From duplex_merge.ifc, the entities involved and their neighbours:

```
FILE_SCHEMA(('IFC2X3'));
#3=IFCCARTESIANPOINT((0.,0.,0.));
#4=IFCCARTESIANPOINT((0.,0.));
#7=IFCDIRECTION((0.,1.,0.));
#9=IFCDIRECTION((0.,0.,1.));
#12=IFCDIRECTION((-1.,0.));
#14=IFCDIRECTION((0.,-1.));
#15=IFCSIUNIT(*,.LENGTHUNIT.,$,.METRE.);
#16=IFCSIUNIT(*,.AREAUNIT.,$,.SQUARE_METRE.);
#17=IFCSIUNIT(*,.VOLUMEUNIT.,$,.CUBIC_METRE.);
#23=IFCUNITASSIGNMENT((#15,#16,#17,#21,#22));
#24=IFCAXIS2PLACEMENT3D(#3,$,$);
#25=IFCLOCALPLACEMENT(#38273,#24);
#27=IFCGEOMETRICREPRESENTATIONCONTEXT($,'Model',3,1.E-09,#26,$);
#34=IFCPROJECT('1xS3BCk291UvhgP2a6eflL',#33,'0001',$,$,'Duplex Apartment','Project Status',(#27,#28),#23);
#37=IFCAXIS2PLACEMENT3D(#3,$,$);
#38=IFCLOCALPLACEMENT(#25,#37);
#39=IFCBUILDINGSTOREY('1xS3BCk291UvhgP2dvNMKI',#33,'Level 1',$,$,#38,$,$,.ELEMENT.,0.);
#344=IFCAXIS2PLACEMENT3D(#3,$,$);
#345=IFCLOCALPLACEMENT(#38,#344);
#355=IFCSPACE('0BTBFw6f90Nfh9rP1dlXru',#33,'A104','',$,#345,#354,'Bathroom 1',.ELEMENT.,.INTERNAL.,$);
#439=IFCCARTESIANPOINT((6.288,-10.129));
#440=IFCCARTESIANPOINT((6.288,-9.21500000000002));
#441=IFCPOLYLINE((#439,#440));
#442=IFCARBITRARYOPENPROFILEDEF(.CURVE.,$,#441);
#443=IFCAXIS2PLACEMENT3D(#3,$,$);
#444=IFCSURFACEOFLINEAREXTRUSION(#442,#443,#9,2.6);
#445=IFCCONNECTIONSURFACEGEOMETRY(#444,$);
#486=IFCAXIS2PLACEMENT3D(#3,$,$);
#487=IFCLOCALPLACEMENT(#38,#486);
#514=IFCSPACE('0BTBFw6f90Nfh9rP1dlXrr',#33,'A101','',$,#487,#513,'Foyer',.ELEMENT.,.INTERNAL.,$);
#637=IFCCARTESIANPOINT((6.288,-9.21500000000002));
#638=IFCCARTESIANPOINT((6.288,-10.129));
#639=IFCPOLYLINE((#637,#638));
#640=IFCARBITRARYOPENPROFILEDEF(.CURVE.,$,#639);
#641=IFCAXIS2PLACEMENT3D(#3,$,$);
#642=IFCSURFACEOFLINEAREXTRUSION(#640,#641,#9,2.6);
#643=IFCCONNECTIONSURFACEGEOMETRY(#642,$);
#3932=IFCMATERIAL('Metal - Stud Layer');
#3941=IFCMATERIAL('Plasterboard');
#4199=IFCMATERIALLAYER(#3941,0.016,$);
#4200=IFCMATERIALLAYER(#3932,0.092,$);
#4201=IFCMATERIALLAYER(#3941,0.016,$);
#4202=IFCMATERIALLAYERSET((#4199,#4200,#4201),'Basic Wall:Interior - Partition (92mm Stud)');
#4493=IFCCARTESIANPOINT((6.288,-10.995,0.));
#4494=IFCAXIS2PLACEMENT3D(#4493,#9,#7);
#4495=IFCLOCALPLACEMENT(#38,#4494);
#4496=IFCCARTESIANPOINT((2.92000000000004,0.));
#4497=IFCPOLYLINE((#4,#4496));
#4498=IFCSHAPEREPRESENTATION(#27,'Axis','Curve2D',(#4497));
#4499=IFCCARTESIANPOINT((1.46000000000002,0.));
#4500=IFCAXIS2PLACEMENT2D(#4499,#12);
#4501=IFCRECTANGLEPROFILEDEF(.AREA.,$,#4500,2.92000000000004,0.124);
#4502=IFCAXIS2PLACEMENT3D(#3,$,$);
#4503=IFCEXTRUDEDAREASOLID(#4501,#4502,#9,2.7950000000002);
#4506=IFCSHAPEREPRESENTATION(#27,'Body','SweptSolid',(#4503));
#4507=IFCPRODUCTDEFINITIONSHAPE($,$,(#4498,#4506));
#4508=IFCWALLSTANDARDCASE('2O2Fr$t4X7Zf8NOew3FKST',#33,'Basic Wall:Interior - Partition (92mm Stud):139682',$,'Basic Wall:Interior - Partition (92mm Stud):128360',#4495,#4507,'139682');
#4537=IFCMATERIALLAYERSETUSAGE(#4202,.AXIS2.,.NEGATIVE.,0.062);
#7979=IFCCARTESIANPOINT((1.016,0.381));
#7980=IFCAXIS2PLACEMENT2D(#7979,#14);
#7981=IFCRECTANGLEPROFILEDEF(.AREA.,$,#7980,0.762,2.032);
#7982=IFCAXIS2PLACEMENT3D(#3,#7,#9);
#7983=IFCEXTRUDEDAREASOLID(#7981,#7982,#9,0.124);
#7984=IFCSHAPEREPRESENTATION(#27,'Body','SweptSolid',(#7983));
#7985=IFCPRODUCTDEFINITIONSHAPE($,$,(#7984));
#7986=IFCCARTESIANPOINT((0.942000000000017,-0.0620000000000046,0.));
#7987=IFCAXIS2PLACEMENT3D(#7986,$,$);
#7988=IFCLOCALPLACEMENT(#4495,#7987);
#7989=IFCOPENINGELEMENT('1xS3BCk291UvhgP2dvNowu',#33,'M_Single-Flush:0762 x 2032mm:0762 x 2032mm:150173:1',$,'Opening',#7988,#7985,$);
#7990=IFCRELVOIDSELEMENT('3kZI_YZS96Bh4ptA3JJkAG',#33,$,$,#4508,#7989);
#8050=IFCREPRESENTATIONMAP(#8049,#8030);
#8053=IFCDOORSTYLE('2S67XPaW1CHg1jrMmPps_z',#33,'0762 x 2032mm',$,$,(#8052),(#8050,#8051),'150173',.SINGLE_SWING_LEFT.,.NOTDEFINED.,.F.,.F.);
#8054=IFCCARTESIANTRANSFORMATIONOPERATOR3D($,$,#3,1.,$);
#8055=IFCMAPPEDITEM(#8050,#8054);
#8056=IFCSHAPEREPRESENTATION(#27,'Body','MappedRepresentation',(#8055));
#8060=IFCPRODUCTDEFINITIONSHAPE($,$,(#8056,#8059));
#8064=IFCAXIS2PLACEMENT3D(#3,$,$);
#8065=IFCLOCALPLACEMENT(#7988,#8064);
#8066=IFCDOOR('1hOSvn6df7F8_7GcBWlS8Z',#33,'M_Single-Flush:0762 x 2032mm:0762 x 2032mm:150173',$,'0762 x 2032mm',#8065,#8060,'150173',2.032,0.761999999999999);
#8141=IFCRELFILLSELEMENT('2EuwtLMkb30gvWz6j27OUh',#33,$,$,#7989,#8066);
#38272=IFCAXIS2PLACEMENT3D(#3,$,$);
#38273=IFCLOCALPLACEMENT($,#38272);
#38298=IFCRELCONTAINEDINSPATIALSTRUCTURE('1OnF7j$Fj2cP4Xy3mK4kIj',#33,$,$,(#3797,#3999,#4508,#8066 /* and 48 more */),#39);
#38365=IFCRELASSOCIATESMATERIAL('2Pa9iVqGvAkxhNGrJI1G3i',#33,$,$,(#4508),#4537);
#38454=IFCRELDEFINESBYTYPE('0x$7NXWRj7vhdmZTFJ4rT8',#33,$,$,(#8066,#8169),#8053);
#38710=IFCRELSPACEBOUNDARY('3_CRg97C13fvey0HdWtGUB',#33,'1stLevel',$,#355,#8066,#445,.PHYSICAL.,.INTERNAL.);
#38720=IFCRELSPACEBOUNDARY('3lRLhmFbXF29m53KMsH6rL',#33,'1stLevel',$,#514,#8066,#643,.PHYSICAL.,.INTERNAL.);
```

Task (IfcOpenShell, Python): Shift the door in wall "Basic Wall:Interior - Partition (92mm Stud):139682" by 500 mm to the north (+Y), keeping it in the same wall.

```python
import numpy as np
import ifcopenshell
import ifcopenshell.api.geometry
import ifcopenshell.util.placement

model = ifcopenshell.open("duplex_merge.ifc")

door = model.by_guid("1hOSvn6df7F8_7GcBWlS8Z")
opening = door.FillsVoids[0].RelatingOpeningElement
wall = opening.VoidsElements[0].RelatingBuildingElement

wall_matrix = ifcopenshell.util.placement.get_local_placement(wall.ObjectPlacement)
shift = wall_matrix[:3, 0] * 0.5
before = ifcopenshell.util.placement.get_local_placement(door.ObjectPlacement)[:3, 3].copy()

# The door is placed relative to its opening, so it follows when the opening moves.
matrix = ifcopenshell.util.placement.get_local_placement(opening.ObjectPlacement)
matrix[:3, 3] += shift
ifcopenshell.api.geometry.edit_object_placement(
    model, product=opening, matrix=matrix, is_si=False, should_transform_children=True
)

# Space boundary surfaces are stored in each space's coordinates; move them too.
for rel in door.ProvidesBoundaries:
    if not rel.ConnectionGeometry:
        continue
    surface = rel.ConnectionGeometry.SurfaceOnRelatingElement
    space_matrix = ifcopenshell.util.placement.get_local_placement(rel.RelatingSpace.ObjectPlacement)
    point = np.array(surface.Position.Location.Coordinates) + space_matrix[:3, :3].T @ shift
    surface.Position = model.createIfcAxis2Placement3D(
        model.createIfcCartesianPoint(point.tolist()), surface.Position.Axis, surface.Position.RefDirection
    )

after = ifcopenshell.util.placement.get_local_placement(door.ObjectPlacement)[:3, 3]
print("door moved by", (after - before).round(3) + 0.0)

model.write("duplex_merge-out.ifc")
```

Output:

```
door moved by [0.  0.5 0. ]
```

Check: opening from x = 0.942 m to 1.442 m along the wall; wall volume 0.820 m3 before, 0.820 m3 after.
